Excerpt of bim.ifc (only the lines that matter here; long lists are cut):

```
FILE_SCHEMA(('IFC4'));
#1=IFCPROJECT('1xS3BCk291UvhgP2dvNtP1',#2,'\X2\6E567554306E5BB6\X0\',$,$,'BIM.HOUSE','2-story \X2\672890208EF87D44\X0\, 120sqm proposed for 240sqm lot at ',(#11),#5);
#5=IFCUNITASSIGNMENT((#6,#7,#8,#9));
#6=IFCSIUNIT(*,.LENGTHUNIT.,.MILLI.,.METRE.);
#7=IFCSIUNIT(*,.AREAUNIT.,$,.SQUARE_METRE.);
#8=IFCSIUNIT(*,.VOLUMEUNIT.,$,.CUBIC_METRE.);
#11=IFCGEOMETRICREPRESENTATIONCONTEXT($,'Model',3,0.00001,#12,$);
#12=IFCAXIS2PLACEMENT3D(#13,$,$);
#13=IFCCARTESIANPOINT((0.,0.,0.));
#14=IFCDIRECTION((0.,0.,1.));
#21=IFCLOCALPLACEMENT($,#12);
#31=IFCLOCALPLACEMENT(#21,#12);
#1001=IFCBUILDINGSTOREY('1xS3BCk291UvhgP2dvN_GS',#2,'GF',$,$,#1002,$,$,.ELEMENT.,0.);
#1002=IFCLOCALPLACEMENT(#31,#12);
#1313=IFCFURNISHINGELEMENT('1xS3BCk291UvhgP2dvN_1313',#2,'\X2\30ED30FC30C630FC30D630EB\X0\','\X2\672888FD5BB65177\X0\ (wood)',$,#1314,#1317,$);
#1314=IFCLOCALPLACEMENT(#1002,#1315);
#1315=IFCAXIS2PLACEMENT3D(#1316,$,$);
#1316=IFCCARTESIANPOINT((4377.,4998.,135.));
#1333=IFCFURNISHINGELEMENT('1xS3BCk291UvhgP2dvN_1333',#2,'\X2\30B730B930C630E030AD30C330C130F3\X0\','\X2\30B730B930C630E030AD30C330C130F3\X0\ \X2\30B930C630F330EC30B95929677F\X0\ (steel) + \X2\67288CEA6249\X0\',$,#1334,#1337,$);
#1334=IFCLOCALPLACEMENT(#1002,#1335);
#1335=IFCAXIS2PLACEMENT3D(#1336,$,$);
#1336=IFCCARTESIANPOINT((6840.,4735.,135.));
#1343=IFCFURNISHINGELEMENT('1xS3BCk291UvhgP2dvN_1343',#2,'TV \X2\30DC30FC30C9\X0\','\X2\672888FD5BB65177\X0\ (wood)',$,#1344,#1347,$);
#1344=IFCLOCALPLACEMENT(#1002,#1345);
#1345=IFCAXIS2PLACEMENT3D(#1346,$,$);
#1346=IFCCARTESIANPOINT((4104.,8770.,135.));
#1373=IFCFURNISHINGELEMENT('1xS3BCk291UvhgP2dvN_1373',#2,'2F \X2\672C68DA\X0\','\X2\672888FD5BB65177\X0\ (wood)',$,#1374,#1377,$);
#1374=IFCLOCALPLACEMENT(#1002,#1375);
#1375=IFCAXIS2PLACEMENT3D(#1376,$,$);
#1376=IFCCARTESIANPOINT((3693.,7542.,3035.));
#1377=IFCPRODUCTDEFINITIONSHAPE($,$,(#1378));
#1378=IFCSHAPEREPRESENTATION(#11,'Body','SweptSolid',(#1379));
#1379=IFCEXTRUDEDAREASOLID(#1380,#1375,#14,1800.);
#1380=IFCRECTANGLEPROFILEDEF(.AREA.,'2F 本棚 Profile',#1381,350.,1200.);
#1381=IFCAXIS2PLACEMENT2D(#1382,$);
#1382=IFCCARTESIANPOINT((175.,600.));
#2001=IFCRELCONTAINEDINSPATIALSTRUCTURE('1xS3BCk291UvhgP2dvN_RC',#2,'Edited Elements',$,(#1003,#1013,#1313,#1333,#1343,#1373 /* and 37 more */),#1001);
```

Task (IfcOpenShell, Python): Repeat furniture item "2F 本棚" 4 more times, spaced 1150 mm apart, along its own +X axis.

```python
import ifcopenshell
import ifcopenshell.api.geometry
import ifcopenshell.api.root
import ifcopenshell.util.element
import ifcopenshell.util.placement

model = ifcopenshell.open("bim.ifc")


def reuse_history(source, copy):
    """copy_class also copies each property set's owner history, people and application; keep the originals."""
    for rel in copy.IsDefinedBy:
        if rel.is_a("IfcRelDefinesByProperties") and (history := rel.RelatingPropertyDefinition.OwnerHistory):
            rel.RelatingPropertyDefinition.OwnerHistory = source.OwnerHistory
            ifcopenshell.util.element.remove_deep2(model, history)


source = model.by_guid("1xS3BCk291UvhgP2dvN_1373")
base = ifcopenshell.util.placement.get_local_placement(source.ObjectPlacement)
step = base[:3, 0] * 1150.0

for i in range(1, 5):
    copy = ifcopenshell.api.root.copy_class(model, product=source)
    copy.Representation = ifcopenshell.util.element.copy_deep(
        model, source.Representation, exclude=["IfcGeometricRepresentationContext", "IfcRepresentationMap"]
    )
    reuse_history(source, copy)
    matrix = base.copy()
    matrix[:3, 3] += i * step
    print("added at", matrix[:3, 3].round(3) + 0.0)
    ifcopenshell.api.geometry.edit_object_placement(model, product=copy, matrix=matrix, is_si=False)

model.write("bim-out.ifc")
```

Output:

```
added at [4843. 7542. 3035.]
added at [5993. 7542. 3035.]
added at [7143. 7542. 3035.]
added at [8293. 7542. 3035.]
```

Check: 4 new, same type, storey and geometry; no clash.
